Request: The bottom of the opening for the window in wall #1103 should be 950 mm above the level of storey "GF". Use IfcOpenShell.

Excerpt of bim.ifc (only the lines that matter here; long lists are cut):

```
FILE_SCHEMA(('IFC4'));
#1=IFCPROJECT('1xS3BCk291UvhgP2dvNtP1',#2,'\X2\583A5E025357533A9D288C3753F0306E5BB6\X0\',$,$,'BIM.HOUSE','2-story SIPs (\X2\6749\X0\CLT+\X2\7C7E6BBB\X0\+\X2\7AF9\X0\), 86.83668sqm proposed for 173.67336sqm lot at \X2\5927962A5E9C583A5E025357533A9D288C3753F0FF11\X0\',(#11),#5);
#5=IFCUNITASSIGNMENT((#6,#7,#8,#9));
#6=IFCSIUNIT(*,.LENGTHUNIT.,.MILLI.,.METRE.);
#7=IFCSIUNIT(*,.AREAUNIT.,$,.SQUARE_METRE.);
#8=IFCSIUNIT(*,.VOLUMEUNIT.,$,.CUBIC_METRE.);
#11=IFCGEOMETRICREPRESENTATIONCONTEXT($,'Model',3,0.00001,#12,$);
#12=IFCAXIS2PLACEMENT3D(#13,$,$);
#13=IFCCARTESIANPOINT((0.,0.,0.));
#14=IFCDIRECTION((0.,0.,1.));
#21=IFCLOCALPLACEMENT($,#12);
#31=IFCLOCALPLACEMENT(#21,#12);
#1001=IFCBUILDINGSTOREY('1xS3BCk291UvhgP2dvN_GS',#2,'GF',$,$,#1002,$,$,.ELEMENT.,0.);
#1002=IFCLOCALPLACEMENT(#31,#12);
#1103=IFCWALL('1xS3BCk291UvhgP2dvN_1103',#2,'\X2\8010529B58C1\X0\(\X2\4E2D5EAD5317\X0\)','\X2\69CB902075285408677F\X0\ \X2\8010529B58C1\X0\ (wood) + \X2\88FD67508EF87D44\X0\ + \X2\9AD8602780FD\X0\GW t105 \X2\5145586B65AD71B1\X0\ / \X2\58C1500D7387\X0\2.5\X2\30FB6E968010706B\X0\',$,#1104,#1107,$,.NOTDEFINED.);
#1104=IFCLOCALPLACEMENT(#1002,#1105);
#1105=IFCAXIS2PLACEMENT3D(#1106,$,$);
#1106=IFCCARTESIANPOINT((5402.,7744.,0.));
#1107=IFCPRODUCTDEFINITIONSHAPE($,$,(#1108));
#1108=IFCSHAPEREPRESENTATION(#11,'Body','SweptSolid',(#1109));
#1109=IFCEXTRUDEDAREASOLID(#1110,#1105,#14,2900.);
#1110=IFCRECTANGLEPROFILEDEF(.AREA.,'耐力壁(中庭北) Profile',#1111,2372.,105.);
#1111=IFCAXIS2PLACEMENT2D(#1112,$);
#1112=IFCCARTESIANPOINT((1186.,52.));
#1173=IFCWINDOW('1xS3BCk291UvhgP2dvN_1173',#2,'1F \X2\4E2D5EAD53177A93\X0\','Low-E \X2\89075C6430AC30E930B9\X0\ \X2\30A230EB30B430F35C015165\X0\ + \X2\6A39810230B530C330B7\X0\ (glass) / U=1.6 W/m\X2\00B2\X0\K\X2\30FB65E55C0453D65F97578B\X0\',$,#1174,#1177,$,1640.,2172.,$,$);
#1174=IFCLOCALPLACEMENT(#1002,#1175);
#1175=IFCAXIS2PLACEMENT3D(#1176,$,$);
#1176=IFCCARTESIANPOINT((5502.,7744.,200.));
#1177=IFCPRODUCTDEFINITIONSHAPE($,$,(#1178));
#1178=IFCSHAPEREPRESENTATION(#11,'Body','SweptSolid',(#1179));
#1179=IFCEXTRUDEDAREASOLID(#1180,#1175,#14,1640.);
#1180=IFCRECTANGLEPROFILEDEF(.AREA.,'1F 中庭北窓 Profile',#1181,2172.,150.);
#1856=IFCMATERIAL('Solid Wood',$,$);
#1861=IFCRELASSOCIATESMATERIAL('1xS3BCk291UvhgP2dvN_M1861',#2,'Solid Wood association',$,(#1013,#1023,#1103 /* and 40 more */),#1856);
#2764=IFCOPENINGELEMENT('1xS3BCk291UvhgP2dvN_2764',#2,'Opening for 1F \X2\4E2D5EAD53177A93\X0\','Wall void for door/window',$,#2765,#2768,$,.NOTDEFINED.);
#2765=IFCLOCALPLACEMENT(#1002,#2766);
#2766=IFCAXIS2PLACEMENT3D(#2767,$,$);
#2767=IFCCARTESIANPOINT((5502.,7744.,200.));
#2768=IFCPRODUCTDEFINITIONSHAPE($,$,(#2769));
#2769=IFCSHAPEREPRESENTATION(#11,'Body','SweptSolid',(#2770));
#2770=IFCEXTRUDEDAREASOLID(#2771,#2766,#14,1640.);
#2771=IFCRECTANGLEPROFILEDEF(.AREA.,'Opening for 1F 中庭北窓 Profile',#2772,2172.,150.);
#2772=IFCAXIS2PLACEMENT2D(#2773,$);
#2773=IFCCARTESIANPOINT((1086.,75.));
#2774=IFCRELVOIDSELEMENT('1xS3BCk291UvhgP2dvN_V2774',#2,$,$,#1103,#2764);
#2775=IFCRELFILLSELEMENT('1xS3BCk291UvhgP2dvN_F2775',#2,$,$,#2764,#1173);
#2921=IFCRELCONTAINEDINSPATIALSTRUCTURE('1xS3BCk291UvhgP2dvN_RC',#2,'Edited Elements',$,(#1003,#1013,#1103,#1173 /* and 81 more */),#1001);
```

```python
import numpy as np
import ifcopenshell
import ifcopenshell.api.geometry
import ifcopenshell.geom
import ifcopenshell.util.element
import ifcopenshell.util.placement
import ifcopenshell.util.shape
import ifcopenshell.util.unit

model = ifcopenshell.open("bim.ifc")
unit_scale = ifcopenshell.util.unit.calculate_unit_scale(model)

window = model.by_id(1173)
opening = window.FillsVoids[0].RelatingOpeningElement
storey = ifcopenshell.util.element.get_container(window, ifc_class="IfcBuildingStorey")
level = ifcopenshell.util.placement.get_local_placement(storey.ObjectPlacement)[2, 3]

# The opening's origin need not be at the sill, so measure its lowest point.
shape = ifcopenshell.geom.create_shape(ifcopenshell.geom.settings(), opening)
bottom = ifcopenshell.util.shape.get_shape_bottom_elevation(shape, shape.geometry) / unit_scale
dz = level + 950.0 - bottom

shift = np.array([0.0, 0.0, dz])
# The window is not placed relative to its opening, so move both.
for product in (opening, window):
    matrix = ifcopenshell.util.placement.get_local_placement(product.ObjectPlacement)
    matrix[:3, 3] += shift
    ifcopenshell.api.geometry.edit_object_placement(model, product=product, matrix=matrix, is_si=False)

print(f"moved by {dz * unit_scale:+.3f} m")

model.write("bim_rev.ifc")
```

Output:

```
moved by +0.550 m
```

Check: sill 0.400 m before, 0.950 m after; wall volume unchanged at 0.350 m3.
